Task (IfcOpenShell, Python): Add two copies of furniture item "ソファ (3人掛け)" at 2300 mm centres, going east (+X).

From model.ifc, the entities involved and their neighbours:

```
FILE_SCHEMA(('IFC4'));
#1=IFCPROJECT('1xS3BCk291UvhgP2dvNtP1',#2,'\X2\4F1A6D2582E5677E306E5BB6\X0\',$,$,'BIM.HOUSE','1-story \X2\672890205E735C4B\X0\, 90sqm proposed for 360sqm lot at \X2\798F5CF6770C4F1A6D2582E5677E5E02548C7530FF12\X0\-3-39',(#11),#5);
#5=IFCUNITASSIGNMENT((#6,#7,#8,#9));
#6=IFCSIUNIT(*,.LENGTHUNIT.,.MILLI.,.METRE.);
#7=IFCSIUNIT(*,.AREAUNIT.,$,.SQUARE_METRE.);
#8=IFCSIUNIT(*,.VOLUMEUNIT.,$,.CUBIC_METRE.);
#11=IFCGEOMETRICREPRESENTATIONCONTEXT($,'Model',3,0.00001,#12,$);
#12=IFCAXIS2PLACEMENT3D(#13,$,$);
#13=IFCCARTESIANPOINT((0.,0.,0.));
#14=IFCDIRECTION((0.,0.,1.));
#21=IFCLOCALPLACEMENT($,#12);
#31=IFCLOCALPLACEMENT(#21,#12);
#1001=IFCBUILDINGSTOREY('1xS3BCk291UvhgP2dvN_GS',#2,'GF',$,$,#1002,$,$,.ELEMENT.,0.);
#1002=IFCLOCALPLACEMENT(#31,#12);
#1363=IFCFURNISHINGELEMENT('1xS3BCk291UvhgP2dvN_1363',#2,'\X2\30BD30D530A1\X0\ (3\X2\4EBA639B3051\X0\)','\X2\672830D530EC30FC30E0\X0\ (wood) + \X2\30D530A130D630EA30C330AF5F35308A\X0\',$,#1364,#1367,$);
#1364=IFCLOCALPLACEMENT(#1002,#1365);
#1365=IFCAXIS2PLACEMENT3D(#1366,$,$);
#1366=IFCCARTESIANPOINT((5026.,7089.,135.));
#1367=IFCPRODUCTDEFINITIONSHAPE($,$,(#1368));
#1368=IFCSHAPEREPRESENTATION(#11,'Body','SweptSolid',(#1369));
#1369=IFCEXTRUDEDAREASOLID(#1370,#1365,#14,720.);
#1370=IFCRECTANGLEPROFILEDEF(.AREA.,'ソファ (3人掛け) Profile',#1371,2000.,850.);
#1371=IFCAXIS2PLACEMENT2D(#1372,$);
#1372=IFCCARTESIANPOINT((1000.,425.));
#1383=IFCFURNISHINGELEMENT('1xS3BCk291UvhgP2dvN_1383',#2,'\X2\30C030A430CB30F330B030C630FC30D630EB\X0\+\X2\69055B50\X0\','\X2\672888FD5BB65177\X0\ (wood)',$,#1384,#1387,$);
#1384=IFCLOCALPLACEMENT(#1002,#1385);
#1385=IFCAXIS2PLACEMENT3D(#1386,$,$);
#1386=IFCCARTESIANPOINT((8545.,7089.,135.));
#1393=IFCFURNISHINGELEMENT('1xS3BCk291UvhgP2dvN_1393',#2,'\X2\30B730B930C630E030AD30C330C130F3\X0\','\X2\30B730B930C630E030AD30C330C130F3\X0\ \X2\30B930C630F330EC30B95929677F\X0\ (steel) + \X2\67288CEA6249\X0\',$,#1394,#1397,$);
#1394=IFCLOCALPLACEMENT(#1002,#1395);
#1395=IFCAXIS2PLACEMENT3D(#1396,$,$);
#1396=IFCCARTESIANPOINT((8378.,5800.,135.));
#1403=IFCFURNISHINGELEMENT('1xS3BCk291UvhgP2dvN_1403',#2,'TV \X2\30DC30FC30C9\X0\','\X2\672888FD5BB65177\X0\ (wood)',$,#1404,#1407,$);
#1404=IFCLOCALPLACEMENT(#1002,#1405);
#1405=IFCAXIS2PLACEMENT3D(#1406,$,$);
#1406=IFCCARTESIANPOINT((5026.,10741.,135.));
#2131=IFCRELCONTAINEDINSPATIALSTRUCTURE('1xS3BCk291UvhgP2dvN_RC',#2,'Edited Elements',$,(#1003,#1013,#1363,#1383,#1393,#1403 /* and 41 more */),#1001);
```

```python
import numpy as np
import ifcopenshell
import ifcopenshell.api.geometry
import ifcopenshell.api.root
import ifcopenshell.util.element
import ifcopenshell.util.placement
import ifcopenshell.util.unit

model = ifcopenshell.open("model.ifc")
unit_scale = ifcopenshell.util.unit.calculate_unit_scale(model)


def reuse_history(source, copy):
    """copy_class also copies each property set's owner history, people and application; keep the originals."""
    for rel in copy.IsDefinedBy:
        if rel.is_a("IfcRelDefinesByProperties") and (history := rel.RelatingPropertyDefinition.OwnerHistory):
            rel.RelatingPropertyDefinition.OwnerHistory = source.OwnerHistory
            ifcopenshell.util.element.remove_deep2(model, history)


source = model.by_guid("1xS3BCk291UvhgP2dvN_1363")
base = ifcopenshell.util.placement.get_local_placement(source.ObjectPlacement)
step = np.array([1.0, 0.0, 0.0]) * 2.3 / unit_scale

for i in range(1, 3):
    copy = ifcopenshell.api.root.copy_class(model, product=source)
    copy.Representation = ifcopenshell.util.element.copy_deep(
        model, source.Representation, exclude=["IfcGeometricRepresentationContext", "IfcRepresentationMap"]
    )
    reuse_history(source, copy)
    matrix = base.copy()
    matrix[:3, 3] += i * step
    print("added at", matrix[:3, 3].round(3) + 0.0)
    ifcopenshell.api.geometry.edit_object_placement(model, product=copy, matrix=matrix, is_si=False)

model.write("model-out.ifc")
```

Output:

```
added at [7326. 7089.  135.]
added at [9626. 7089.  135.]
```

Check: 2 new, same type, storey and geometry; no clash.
